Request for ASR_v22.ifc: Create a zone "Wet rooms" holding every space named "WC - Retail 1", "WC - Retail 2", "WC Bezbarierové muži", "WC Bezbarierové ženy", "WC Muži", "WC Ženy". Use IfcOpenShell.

First a look at what the model holds.

```python
import ifcopenshell

model = ifcopenshell.open("ASR_v22.ifc")
print(model.schema)
seen = {}
for space in model.by_type("IfcSpace"):
    seen[space.LongName] = seen.get(space.LongName, 0) + 1
for name, count in sorted(seen.items(), key=str):
    print(count, "x", name)
print("zones:", [z.Name for z in model.by_type("IfcZone")][:20])
```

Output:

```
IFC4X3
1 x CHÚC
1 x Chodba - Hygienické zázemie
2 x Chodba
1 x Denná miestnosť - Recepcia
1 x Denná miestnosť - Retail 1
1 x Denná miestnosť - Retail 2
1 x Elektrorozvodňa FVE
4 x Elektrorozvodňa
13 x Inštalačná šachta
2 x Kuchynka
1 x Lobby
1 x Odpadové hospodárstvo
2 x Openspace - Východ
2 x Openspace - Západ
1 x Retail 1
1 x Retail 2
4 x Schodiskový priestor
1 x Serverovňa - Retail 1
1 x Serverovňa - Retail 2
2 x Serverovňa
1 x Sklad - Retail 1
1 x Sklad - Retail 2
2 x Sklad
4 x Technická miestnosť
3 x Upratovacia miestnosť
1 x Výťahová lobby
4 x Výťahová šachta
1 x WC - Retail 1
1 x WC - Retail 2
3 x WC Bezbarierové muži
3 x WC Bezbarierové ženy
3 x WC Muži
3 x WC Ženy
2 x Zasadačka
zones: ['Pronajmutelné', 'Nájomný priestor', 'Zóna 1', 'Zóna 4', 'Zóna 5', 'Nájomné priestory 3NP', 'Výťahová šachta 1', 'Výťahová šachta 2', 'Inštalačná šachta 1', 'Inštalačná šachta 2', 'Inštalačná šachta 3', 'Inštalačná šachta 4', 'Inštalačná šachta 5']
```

```python
import ifcopenshell
import ifcopenshell.api.group
import ifcopenshell.api.root

model = ifcopenshell.open("ASR_v22.ifc")

names = {"WC - Retail 1", "WC - Retail 2", "WC Bezbarierové muži", "WC Bezbarierové ženy", "WC Muži", "WC Ženy"}
spaces = [s for s in model.by_type("IfcSpace") if s.LongName in names]

zone = ifcopenshell.api.root.create_entity(model, ifc_class="IfcZone", name="Wet rooms")
ifcopenshell.api.group.assign_group(model, products=spaces, group=zone)
print(len(spaces), "spaces in", zone.Name)

model.write("ASR_v22_v2.ifc")
```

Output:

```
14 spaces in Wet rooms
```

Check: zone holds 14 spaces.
